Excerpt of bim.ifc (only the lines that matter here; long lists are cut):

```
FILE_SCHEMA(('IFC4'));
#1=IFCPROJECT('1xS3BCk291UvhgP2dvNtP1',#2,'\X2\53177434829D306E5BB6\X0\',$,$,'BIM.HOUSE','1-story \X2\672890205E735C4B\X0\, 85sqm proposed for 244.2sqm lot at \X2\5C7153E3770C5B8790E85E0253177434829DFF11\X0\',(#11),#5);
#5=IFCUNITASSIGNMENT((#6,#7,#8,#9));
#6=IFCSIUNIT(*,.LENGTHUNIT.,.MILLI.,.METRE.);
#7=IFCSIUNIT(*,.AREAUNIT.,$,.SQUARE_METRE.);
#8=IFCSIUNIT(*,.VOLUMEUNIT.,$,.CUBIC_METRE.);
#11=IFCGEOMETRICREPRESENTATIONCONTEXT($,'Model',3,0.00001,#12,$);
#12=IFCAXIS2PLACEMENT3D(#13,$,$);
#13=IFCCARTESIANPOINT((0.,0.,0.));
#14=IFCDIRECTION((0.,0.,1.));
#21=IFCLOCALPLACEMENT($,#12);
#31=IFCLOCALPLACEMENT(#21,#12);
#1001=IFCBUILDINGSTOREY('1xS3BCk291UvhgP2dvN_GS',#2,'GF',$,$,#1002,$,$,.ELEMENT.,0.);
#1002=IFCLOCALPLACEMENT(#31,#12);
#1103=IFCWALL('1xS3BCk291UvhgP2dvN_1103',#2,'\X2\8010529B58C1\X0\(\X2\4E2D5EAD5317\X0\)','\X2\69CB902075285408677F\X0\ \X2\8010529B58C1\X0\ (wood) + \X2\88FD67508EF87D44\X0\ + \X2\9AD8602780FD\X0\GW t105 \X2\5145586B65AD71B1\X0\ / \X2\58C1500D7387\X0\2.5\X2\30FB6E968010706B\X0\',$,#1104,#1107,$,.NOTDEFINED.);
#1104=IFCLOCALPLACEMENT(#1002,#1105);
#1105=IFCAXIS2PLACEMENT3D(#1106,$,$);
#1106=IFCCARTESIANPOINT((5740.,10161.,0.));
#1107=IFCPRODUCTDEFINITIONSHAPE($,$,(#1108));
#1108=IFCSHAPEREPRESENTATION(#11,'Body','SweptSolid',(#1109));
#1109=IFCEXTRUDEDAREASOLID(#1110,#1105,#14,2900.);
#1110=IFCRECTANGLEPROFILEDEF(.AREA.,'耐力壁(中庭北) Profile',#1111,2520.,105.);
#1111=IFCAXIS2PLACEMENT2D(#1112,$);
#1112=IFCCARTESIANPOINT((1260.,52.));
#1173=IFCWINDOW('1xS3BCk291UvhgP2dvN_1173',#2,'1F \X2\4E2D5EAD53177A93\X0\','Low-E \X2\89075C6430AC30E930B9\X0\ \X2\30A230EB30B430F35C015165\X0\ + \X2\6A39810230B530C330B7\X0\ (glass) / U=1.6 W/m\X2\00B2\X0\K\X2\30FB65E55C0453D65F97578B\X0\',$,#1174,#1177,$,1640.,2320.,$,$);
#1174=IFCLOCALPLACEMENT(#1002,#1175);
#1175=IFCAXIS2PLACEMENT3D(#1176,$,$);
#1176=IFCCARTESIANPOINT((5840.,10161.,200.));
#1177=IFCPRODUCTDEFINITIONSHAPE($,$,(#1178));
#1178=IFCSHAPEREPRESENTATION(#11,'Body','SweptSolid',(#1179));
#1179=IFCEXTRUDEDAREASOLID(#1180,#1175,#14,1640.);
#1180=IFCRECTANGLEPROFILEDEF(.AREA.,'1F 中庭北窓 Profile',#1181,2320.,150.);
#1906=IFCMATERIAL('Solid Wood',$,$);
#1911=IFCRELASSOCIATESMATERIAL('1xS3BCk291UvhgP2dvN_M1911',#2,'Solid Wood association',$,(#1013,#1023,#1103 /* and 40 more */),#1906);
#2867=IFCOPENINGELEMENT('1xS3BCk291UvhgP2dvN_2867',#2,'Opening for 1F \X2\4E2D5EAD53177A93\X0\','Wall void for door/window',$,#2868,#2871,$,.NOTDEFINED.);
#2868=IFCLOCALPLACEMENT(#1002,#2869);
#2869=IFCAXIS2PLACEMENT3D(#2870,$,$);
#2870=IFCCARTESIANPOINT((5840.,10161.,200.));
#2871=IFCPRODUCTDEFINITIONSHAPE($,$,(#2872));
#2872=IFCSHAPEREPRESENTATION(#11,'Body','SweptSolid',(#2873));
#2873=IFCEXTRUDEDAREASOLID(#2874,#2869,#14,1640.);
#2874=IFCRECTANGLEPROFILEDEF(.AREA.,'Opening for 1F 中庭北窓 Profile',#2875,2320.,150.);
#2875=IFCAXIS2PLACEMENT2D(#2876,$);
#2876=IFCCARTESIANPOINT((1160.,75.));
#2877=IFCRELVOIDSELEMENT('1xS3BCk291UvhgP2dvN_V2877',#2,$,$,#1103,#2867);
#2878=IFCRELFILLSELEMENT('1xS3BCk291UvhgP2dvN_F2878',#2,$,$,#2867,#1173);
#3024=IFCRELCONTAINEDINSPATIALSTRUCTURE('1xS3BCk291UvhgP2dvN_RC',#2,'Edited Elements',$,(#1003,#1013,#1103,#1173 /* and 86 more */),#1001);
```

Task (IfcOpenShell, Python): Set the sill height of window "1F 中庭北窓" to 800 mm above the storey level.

```python
import numpy as np
import ifcopenshell
import ifcopenshell.api.geometry
import ifcopenshell.geom
import ifcopenshell.util.element
import ifcopenshell.util.placement
import ifcopenshell.util.shape
import ifcopenshell.util.unit

model = ifcopenshell.open("bim.ifc")
unit_scale = ifcopenshell.util.unit.calculate_unit_scale(model)

window = model.by_id(1173)
opening = window.FillsVoids[0].RelatingOpeningElement
storey = ifcopenshell.util.element.get_container(window, ifc_class="IfcBuildingStorey")
level = ifcopenshell.util.placement.get_local_placement(storey.ObjectPlacement)[2, 3]

# The opening's origin need not be at the sill, so measure its lowest point.
shape = ifcopenshell.geom.create_shape(ifcopenshell.geom.settings(), opening)
bottom = ifcopenshell.util.shape.get_shape_bottom_elevation(shape, shape.geometry) / unit_scale
dz = level + 0.8 / unit_scale - bottom

shift = np.array([0.0, 0.0, dz])
# The window is not placed relative to its opening, so move both.
for product in (opening, window):
    matrix = ifcopenshell.util.placement.get_local_placement(product.ObjectPlacement)
    matrix[:3, 3] += shift
    ifcopenshell.api.geometry.edit_object_placement(model, product=product, matrix=matrix, is_si=False)

print(f"moved by {dz * unit_scale:+.3f} m")

model.write("bim_rev.ifc")
```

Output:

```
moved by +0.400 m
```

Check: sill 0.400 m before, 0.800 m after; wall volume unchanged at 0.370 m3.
